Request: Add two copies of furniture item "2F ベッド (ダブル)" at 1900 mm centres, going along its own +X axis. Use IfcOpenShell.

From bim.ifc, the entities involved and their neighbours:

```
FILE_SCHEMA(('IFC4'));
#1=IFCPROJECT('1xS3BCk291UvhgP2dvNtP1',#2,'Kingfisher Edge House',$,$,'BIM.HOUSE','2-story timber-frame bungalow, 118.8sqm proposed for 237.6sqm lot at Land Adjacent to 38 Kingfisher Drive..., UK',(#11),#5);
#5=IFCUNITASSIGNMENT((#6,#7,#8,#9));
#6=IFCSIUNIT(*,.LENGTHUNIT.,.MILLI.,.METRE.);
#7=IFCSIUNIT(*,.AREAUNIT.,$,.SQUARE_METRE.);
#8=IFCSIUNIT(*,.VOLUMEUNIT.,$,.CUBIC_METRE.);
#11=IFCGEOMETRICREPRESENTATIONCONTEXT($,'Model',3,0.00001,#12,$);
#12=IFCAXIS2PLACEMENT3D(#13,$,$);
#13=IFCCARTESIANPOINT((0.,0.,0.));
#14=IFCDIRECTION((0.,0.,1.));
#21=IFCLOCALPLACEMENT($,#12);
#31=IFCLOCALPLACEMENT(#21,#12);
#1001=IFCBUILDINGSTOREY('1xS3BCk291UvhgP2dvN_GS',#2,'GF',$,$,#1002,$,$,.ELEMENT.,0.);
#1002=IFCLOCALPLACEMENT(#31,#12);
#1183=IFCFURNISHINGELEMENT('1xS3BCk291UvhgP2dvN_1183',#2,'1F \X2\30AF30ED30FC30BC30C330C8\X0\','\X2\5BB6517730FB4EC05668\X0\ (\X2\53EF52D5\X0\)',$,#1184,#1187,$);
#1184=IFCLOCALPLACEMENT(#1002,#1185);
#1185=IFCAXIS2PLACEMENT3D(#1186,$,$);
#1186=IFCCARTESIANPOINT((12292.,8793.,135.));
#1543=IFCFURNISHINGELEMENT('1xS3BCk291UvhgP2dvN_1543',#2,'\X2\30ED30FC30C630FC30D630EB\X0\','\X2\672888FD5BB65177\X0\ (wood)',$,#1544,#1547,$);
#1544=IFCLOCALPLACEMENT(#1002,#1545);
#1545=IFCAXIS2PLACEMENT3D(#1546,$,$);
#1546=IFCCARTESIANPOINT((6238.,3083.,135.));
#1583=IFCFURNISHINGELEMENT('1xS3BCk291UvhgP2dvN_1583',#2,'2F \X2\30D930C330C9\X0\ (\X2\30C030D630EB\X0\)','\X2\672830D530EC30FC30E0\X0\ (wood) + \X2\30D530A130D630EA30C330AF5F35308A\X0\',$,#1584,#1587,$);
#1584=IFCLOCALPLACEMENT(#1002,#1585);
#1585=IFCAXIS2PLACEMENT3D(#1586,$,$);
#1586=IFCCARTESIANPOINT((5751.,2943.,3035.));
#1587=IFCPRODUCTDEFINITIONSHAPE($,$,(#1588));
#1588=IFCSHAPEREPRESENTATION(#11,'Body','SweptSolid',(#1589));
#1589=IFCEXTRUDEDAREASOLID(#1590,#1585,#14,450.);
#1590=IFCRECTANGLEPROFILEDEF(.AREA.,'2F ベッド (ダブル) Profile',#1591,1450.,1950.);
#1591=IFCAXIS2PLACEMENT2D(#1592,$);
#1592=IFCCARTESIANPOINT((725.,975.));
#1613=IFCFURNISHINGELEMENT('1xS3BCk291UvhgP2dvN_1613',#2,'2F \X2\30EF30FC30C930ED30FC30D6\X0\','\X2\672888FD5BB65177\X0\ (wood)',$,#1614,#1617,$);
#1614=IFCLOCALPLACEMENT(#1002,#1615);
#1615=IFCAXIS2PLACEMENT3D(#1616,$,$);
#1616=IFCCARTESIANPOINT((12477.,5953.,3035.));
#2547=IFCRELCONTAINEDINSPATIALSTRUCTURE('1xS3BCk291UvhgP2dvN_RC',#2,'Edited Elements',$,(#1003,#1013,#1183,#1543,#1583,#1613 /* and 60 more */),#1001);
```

```python
import ifcopenshell
import ifcopenshell.api.geometry
import ifcopenshell.api.root
import ifcopenshell.util.element
import ifcopenshell.util.placement

model = ifcopenshell.open("bim.ifc")


def reuse_history(source, copy):
    """copy_class also copies each property set's owner history, people and application; keep the originals."""
    for rel in copy.IsDefinedBy:
        if rel.is_a("IfcRelDefinesByProperties") and (history := rel.RelatingPropertyDefinition.OwnerHistory):
            rel.RelatingPropertyDefinition.OwnerHistory = source.OwnerHistory
            ifcopenshell.util.element.remove_deep2(model, history)


source = model.by_guid("1xS3BCk291UvhgP2dvN_1583")
base = ifcopenshell.util.placement.get_local_placement(source.ObjectPlacement)
step = base[:3, 0] * 1900.0

for i in range(1, 3):
    copy = ifcopenshell.api.root.copy_class(model, product=source)
    copy.Representation = ifcopenshell.util.element.copy_deep(
        model, source.Representation, exclude=["IfcGeometricRepresentationContext", "IfcRepresentationMap"]
    )
    reuse_history(source, copy)
    matrix = base.copy()
    matrix[:3, 3] += i * step
    print("added at", matrix[:3, 3].round(3) + 0.0)
    ifcopenshell.api.geometry.edit_object_placement(model, product=copy, matrix=matrix, is_si=False)

model.write("bim_updated.ifc")
```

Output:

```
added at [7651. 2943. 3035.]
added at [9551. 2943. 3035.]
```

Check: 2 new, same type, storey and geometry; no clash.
